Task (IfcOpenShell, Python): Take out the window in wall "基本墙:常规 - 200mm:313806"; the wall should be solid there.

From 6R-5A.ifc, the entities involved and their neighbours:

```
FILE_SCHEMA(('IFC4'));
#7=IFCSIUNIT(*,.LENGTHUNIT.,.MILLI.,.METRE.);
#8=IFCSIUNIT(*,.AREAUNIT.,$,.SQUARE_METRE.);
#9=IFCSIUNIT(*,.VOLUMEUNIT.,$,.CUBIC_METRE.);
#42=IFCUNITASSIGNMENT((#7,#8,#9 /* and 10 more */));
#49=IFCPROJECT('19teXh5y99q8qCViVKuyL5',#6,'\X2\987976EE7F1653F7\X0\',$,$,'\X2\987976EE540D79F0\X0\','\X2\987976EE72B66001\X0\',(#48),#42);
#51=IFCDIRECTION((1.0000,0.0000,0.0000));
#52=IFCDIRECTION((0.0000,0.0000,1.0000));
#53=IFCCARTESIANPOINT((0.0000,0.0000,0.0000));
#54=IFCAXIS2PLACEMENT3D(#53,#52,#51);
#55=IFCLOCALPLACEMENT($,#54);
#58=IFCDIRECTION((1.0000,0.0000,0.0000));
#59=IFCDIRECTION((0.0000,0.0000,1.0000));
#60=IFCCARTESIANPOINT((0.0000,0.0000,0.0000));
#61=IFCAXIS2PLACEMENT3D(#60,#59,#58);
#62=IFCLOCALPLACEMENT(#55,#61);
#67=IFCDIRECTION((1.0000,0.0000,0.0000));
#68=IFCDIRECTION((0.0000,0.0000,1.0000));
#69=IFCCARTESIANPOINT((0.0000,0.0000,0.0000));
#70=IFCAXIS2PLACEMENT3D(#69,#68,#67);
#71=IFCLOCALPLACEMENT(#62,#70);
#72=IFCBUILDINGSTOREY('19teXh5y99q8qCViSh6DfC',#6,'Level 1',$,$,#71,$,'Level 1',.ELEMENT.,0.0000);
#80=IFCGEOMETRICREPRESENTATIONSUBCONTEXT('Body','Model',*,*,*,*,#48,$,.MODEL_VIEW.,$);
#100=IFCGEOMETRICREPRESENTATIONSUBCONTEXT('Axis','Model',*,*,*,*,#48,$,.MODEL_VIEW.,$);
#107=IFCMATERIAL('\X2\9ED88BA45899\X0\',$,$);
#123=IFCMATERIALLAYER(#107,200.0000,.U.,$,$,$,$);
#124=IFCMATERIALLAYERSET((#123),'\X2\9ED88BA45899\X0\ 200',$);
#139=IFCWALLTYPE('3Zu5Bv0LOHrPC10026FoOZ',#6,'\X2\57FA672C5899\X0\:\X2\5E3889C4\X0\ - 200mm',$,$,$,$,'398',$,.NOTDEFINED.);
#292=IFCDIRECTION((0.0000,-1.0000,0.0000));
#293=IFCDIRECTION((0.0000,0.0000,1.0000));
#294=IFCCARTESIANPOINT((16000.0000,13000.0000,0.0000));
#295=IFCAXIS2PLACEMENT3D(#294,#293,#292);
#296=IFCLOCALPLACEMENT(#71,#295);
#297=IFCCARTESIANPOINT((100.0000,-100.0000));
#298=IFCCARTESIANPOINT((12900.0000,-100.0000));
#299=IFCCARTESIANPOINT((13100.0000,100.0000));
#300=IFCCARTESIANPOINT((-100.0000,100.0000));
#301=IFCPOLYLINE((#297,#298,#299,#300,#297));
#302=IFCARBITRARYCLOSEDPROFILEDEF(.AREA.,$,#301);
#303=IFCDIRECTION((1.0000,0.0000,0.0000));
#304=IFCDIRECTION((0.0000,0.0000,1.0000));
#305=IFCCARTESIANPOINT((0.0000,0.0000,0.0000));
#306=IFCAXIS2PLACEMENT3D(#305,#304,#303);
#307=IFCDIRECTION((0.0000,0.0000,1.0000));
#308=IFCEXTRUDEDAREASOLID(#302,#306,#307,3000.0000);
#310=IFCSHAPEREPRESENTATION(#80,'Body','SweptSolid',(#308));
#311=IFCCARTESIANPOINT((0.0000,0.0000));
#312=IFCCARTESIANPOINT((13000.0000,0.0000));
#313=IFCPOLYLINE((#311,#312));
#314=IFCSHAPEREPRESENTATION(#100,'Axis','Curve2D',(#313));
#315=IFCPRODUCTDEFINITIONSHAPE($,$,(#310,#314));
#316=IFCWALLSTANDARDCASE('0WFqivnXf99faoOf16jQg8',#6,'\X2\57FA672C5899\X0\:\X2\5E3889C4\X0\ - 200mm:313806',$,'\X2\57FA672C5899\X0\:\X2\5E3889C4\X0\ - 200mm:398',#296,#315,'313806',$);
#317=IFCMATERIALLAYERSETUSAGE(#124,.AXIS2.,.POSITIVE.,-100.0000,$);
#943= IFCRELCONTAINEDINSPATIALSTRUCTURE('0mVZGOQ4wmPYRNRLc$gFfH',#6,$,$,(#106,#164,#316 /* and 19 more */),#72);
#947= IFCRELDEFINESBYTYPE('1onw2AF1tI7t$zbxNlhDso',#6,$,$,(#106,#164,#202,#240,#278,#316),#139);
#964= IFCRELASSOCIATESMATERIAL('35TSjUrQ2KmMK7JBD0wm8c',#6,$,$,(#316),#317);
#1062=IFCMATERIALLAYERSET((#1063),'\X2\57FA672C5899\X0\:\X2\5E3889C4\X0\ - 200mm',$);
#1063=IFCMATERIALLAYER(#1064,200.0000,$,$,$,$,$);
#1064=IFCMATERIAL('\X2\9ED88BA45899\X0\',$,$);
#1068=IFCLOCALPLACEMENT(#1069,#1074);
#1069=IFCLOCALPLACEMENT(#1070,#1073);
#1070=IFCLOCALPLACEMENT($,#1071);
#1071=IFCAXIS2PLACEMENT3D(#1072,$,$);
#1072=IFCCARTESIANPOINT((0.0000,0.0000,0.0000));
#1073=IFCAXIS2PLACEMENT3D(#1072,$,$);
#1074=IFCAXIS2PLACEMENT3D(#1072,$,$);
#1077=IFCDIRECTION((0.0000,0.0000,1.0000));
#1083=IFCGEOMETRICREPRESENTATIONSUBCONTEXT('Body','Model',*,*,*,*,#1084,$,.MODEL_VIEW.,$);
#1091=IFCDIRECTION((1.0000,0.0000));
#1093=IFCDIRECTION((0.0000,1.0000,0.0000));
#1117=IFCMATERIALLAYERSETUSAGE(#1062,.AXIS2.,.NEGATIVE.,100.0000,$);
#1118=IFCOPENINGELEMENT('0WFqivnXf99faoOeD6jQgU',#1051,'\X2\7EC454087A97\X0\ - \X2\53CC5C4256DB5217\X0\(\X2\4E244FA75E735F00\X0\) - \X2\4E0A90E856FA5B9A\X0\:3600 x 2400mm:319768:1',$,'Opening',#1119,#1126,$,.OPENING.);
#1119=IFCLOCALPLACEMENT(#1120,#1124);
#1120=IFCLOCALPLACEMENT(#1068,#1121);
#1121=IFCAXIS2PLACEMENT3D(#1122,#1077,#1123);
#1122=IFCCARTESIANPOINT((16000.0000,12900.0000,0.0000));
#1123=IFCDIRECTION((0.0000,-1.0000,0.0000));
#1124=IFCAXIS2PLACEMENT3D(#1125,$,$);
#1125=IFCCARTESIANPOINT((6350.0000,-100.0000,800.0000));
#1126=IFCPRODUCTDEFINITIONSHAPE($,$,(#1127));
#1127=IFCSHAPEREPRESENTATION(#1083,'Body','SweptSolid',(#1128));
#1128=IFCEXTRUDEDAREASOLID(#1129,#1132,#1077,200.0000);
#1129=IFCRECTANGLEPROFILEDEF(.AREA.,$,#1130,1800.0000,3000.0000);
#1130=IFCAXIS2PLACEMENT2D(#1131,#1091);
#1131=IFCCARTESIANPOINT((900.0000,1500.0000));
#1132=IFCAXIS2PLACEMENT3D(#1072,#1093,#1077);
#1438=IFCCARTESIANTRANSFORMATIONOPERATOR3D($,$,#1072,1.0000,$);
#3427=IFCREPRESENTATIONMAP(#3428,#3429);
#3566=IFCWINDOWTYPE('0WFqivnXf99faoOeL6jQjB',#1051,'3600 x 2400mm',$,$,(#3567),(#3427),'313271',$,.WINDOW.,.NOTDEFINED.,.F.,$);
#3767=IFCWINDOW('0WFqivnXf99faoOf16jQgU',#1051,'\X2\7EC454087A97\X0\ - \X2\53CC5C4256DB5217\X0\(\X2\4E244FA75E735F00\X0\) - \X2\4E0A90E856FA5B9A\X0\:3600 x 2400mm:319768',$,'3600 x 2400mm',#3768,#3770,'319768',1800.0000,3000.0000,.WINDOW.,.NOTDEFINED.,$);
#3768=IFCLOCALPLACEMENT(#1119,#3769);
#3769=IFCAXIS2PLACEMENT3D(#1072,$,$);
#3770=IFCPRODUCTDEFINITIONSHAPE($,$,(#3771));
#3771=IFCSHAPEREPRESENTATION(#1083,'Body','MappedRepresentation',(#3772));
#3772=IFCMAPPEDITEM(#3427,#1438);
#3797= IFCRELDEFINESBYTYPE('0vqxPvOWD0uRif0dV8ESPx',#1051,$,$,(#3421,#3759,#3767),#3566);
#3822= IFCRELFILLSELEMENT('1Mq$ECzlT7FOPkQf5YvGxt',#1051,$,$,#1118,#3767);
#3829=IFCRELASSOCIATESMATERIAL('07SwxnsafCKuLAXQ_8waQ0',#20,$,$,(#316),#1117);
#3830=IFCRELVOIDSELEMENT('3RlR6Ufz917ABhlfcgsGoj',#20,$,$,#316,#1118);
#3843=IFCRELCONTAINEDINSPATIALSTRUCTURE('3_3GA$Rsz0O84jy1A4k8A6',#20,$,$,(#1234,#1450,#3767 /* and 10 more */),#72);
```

```python
import ifcopenshell
import ifcopenshell.api.feature
import ifcopenshell.api.root
import ifcopenshell.geom
import ifcopenshell.util.shape

model = ifcopenshell.open("6R-5A.ifc")
settings = ifcopenshell.geom.settings()


def volume(element):
    """Net volume in cubic metres, openings subtracted."""
    shape = ifcopenshell.geom.create_shape(settings, element)
    return ifcopenshell.util.shape.get_volume(shape.geometry)


window = model.by_guid("0WFqivnXf99faoOf16jQgU")
opening = window.FillsVoids[0].RelatingOpeningElement
wall = opening.VoidsElements[0].RelatingBuildingElement
before = volume(wall)

ifcopenshell.api.root.remove_product(model, product=window)
ifcopenshell.api.feature.remove_feature(model, feature=opening)

after = volume(wall)

print(f"wall volume {before:.3f} -> {after:.3f} m3")

model.write("6R-5A_v2.ifc")
```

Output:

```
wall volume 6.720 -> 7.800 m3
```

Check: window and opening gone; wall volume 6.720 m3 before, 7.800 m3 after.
